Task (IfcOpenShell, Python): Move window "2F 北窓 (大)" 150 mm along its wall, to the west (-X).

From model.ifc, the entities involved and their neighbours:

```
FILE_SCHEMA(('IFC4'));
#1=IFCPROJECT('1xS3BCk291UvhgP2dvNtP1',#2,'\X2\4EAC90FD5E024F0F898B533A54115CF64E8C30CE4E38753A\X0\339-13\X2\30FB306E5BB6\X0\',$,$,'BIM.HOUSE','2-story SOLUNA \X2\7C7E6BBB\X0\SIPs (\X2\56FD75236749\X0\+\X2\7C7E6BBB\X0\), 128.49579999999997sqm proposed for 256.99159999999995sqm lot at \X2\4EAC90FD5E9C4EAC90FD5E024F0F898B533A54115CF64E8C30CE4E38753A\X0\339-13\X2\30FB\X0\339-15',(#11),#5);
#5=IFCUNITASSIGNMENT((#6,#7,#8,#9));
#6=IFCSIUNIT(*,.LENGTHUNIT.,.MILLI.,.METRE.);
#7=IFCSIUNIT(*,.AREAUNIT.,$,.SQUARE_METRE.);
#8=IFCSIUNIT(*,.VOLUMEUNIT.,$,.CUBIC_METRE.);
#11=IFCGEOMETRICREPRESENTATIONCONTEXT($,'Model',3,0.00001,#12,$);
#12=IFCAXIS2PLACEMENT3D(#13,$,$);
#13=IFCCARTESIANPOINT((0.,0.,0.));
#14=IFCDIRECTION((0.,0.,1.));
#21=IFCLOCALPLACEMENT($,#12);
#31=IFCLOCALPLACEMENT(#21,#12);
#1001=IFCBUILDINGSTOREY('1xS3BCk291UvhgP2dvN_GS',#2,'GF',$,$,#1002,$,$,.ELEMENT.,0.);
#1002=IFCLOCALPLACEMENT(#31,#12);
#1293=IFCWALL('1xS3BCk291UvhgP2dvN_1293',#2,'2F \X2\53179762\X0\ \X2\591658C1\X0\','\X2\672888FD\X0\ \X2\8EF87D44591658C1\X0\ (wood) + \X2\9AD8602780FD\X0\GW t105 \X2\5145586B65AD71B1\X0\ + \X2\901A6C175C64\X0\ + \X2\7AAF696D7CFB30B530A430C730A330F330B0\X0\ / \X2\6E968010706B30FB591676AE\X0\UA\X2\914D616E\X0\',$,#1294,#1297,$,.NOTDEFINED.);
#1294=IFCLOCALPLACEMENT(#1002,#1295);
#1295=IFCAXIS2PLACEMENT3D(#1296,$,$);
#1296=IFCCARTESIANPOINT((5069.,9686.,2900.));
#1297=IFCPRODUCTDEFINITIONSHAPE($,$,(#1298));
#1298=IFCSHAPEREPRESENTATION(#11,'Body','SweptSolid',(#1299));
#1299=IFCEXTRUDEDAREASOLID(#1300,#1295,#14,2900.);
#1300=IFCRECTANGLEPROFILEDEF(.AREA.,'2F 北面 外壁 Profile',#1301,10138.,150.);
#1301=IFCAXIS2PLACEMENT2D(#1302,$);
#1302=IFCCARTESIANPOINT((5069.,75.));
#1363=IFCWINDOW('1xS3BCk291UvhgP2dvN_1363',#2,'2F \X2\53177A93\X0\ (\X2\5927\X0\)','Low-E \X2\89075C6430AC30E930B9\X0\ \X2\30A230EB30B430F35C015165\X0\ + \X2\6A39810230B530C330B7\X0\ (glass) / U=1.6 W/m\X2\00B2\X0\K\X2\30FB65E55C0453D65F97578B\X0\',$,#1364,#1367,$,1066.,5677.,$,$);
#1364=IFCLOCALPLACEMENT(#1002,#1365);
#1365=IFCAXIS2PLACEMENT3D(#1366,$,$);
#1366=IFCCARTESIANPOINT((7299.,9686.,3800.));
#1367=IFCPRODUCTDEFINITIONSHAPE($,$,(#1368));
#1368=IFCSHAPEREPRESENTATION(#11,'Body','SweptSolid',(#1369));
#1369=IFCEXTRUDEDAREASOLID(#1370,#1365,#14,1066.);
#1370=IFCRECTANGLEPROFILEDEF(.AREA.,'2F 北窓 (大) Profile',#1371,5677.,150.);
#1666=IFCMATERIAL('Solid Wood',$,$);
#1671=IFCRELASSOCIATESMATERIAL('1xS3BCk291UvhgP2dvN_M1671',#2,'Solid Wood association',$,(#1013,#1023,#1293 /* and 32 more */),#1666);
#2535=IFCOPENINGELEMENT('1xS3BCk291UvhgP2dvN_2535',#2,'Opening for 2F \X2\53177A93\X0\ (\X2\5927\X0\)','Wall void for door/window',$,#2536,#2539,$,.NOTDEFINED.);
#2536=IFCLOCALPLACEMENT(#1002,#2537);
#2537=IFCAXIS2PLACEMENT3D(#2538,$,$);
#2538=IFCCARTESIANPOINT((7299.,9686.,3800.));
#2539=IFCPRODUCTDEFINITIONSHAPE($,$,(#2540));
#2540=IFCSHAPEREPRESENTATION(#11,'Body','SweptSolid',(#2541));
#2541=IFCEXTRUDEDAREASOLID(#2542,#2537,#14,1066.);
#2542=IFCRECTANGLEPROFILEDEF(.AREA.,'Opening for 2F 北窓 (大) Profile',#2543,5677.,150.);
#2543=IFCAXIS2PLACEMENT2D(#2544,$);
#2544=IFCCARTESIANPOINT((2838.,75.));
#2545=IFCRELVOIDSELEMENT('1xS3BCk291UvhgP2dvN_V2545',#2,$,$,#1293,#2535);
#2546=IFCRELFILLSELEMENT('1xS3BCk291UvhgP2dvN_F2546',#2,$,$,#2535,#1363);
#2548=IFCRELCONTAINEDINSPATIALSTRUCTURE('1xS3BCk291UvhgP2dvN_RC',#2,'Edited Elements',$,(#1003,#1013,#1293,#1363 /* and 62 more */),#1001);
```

```python
import ifcopenshell
import ifcopenshell.api.geometry
import ifcopenshell.util.placement

model = ifcopenshell.open("model.ifc")

window = model.by_id(1363)
opening = window.FillsVoids[0].RelatingOpeningElement
wall = opening.VoidsElements[0].RelatingBuildingElement

wall_matrix = ifcopenshell.util.placement.get_local_placement(wall.ObjectPlacement)
shift = wall_matrix[:3, 0] * -150.0
before = ifcopenshell.util.placement.get_local_placement(window.ObjectPlacement)[:3, 3].copy()

# The window is not placed relative to its opening, so move both.
for product in (opening, window):
    matrix = ifcopenshell.util.placement.get_local_placement(product.ObjectPlacement)
    matrix[:3, 3] += shift
    ifcopenshell.api.geometry.edit_object_placement(model, product=product, matrix=matrix, is_si=False)

after = ifcopenshell.util.placement.get_local_placement(window.ObjectPlacement)[:3, 3]
print("window moved by", (after - before).round(3) + 0.0)

model.write("model_updated.ifc")
```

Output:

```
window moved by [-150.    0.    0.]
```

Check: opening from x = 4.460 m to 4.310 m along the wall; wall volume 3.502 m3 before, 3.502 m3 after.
